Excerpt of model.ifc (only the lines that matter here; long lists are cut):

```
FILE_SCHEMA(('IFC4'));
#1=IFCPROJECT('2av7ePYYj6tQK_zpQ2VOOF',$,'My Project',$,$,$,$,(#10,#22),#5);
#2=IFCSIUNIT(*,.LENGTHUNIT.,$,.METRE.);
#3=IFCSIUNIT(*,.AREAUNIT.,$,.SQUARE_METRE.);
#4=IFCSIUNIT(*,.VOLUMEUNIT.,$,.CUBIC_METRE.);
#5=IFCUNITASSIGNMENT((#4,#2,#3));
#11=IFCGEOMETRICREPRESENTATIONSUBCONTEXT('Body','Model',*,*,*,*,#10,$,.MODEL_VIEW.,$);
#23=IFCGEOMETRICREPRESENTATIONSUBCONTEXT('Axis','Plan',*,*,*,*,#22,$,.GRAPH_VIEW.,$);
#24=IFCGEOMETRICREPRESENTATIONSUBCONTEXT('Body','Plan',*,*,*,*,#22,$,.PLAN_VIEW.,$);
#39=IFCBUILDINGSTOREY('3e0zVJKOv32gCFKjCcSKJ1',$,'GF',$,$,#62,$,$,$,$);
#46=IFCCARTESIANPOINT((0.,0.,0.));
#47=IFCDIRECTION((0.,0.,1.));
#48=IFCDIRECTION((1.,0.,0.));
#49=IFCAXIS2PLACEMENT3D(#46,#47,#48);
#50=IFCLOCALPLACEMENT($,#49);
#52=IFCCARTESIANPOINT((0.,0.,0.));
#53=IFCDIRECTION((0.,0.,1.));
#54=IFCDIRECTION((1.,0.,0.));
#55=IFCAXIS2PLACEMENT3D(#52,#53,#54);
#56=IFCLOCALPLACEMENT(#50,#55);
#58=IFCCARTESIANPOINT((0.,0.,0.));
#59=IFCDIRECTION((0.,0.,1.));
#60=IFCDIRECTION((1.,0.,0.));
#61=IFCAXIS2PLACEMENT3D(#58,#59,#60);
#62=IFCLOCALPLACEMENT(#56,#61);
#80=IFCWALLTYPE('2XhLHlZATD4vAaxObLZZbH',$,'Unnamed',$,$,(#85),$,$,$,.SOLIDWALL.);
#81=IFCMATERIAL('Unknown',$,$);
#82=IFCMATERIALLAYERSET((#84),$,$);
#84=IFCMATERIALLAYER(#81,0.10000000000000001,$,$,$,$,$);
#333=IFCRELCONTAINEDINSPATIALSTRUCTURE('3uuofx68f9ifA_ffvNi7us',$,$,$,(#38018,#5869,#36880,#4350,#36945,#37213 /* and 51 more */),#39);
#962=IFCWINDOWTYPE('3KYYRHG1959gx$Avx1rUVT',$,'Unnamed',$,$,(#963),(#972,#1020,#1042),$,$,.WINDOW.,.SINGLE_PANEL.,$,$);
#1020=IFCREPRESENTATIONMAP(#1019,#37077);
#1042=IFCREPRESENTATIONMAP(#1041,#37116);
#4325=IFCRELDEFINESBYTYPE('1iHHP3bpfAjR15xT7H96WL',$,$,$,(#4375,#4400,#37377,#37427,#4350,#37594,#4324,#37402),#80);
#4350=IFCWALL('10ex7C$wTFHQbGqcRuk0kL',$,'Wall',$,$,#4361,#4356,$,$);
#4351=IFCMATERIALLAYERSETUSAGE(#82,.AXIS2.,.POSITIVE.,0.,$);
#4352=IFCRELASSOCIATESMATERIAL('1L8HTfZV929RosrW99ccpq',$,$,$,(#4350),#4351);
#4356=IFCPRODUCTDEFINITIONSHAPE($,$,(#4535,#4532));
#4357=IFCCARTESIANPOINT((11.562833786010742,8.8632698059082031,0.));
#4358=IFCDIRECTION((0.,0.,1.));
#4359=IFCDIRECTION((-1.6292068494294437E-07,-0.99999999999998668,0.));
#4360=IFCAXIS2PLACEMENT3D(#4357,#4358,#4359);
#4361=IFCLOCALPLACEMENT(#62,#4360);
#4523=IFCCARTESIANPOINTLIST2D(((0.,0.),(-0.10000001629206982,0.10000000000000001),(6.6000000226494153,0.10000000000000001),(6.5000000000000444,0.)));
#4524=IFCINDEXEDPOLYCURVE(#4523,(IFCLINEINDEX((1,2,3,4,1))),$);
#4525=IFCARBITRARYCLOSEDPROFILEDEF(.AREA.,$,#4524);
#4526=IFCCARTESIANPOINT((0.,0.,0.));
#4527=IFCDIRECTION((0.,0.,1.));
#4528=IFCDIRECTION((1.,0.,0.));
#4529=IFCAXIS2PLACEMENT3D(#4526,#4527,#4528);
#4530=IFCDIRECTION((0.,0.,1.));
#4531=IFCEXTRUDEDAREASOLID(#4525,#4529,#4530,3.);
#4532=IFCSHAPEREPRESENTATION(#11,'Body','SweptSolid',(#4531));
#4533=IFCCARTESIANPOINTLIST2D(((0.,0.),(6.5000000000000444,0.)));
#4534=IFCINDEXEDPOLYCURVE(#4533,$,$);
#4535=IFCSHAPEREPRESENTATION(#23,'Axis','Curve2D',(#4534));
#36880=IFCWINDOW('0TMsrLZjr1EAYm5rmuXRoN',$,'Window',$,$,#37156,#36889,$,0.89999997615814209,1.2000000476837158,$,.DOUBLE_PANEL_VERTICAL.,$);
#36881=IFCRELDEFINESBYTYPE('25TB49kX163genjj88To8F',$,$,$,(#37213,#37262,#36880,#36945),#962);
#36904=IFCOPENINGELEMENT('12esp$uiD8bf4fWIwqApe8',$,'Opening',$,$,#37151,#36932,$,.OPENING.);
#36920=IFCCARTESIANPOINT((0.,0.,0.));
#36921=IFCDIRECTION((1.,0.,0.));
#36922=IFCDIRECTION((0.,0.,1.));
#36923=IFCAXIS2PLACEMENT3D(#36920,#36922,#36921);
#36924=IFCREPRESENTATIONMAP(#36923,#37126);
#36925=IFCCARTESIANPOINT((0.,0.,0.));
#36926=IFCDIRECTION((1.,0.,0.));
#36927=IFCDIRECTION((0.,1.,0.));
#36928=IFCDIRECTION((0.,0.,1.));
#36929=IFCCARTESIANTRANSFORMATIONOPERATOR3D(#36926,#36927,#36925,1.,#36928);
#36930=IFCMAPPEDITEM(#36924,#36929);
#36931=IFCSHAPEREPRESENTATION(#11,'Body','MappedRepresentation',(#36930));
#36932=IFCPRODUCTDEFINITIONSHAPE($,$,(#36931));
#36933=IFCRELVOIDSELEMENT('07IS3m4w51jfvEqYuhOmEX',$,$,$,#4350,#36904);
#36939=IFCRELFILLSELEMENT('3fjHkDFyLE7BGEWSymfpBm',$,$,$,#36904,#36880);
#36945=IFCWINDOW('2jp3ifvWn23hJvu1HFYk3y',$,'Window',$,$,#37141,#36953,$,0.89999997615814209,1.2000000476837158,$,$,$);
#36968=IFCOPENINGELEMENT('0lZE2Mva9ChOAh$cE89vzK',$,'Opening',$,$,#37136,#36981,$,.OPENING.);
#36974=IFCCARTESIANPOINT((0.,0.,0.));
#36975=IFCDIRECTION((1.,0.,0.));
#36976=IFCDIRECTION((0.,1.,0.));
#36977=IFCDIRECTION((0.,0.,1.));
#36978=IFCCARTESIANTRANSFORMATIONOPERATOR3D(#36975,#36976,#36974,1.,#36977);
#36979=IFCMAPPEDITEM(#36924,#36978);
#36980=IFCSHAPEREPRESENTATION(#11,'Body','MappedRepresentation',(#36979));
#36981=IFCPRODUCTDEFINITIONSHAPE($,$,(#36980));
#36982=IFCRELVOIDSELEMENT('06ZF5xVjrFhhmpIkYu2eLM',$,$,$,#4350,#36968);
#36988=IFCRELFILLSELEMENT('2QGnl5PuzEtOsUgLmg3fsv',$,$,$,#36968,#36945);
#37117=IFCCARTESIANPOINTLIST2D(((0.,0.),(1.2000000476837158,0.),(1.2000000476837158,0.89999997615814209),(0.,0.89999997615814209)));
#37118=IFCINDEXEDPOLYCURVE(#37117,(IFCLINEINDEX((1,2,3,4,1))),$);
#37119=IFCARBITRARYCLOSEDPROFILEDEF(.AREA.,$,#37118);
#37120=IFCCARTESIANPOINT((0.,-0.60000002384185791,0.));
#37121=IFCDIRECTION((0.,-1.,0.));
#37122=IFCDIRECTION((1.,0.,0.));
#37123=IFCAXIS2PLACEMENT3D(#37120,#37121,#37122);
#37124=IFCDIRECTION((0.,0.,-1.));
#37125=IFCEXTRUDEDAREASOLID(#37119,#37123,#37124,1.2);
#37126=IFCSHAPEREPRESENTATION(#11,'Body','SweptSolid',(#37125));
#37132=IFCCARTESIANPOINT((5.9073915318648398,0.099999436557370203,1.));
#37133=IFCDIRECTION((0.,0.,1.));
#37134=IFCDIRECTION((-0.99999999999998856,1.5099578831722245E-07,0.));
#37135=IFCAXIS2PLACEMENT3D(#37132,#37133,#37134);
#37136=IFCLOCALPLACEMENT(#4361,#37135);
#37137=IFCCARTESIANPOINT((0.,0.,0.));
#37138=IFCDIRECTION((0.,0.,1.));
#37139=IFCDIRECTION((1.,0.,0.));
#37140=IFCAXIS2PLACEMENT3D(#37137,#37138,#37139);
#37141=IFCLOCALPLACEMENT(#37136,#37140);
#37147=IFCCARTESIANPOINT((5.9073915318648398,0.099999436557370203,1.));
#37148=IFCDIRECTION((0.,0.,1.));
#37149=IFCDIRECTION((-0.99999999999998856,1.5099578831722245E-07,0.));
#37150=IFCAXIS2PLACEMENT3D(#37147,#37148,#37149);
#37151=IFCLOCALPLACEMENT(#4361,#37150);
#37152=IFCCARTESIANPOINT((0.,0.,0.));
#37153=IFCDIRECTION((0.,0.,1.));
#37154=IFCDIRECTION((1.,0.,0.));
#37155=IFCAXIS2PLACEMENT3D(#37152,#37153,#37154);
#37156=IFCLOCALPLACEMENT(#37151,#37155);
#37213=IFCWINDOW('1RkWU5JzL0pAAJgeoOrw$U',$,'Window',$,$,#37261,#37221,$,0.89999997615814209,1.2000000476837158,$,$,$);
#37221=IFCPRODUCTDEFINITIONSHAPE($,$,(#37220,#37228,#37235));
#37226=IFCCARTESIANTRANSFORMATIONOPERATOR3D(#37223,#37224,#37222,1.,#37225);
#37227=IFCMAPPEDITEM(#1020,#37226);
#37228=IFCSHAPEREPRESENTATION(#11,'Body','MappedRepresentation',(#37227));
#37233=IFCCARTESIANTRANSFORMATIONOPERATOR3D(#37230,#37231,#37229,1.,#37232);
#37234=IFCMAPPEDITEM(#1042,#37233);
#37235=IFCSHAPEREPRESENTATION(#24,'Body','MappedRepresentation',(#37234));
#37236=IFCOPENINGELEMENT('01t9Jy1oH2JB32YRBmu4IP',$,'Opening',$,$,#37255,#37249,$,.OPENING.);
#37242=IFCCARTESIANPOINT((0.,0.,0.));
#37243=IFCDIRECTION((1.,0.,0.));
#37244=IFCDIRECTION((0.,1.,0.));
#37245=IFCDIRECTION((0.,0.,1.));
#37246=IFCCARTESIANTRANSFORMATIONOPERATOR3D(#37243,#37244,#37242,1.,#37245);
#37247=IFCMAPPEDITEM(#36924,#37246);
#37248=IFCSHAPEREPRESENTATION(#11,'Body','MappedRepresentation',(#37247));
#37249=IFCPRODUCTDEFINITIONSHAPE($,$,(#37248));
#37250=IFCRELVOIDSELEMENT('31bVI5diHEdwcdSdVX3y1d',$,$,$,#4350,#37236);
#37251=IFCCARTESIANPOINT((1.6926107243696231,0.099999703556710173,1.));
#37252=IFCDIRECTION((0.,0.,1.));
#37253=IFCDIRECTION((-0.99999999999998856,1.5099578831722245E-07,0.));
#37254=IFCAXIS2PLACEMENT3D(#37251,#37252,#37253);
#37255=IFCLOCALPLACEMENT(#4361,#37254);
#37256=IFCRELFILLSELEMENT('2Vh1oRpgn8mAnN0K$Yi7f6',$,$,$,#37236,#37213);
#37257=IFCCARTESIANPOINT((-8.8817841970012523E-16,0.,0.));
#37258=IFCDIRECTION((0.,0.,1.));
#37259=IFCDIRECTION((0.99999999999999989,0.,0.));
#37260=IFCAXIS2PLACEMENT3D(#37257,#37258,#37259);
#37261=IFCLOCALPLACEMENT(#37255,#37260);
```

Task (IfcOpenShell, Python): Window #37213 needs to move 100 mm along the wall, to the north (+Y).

```python
import ifcopenshell
import ifcopenshell.api.geometry
import ifcopenshell.util.placement
import ifcopenshell.util.unit

model = ifcopenshell.open("model.ifc")
unit_scale = ifcopenshell.util.unit.calculate_unit_scale(model)

window = model.by_guid("1RkWU5JzL0pAAJgeoOrw$U")
opening = window.FillsVoids[0].RelatingOpeningElement
wall = opening.VoidsElements[0].RelatingBuildingElement

wall_matrix = ifcopenshell.util.placement.get_local_placement(wall.ObjectPlacement)
shift = wall_matrix[:3, 0] * -0.1 / unit_scale
before = ifcopenshell.util.placement.get_local_placement(window.ObjectPlacement)[:3, 3].copy()

# The window is placed relative to its opening, so it follows when the opening moves.
matrix = ifcopenshell.util.placement.get_local_placement(opening.ObjectPlacement)
matrix[:3, 3] += shift
ifcopenshell.api.geometry.edit_object_placement(
    model, product=opening, matrix=matrix, is_si=False, should_transform_children=True
)

after = ifcopenshell.util.placement.get_local_placement(window.ObjectPlacement)[:3, 3]
print("window moved by", (after - before).round(3) + 0.0)

model.write("model-out.ifc")
```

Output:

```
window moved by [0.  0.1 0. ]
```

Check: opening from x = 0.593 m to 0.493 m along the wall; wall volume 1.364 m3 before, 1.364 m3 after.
